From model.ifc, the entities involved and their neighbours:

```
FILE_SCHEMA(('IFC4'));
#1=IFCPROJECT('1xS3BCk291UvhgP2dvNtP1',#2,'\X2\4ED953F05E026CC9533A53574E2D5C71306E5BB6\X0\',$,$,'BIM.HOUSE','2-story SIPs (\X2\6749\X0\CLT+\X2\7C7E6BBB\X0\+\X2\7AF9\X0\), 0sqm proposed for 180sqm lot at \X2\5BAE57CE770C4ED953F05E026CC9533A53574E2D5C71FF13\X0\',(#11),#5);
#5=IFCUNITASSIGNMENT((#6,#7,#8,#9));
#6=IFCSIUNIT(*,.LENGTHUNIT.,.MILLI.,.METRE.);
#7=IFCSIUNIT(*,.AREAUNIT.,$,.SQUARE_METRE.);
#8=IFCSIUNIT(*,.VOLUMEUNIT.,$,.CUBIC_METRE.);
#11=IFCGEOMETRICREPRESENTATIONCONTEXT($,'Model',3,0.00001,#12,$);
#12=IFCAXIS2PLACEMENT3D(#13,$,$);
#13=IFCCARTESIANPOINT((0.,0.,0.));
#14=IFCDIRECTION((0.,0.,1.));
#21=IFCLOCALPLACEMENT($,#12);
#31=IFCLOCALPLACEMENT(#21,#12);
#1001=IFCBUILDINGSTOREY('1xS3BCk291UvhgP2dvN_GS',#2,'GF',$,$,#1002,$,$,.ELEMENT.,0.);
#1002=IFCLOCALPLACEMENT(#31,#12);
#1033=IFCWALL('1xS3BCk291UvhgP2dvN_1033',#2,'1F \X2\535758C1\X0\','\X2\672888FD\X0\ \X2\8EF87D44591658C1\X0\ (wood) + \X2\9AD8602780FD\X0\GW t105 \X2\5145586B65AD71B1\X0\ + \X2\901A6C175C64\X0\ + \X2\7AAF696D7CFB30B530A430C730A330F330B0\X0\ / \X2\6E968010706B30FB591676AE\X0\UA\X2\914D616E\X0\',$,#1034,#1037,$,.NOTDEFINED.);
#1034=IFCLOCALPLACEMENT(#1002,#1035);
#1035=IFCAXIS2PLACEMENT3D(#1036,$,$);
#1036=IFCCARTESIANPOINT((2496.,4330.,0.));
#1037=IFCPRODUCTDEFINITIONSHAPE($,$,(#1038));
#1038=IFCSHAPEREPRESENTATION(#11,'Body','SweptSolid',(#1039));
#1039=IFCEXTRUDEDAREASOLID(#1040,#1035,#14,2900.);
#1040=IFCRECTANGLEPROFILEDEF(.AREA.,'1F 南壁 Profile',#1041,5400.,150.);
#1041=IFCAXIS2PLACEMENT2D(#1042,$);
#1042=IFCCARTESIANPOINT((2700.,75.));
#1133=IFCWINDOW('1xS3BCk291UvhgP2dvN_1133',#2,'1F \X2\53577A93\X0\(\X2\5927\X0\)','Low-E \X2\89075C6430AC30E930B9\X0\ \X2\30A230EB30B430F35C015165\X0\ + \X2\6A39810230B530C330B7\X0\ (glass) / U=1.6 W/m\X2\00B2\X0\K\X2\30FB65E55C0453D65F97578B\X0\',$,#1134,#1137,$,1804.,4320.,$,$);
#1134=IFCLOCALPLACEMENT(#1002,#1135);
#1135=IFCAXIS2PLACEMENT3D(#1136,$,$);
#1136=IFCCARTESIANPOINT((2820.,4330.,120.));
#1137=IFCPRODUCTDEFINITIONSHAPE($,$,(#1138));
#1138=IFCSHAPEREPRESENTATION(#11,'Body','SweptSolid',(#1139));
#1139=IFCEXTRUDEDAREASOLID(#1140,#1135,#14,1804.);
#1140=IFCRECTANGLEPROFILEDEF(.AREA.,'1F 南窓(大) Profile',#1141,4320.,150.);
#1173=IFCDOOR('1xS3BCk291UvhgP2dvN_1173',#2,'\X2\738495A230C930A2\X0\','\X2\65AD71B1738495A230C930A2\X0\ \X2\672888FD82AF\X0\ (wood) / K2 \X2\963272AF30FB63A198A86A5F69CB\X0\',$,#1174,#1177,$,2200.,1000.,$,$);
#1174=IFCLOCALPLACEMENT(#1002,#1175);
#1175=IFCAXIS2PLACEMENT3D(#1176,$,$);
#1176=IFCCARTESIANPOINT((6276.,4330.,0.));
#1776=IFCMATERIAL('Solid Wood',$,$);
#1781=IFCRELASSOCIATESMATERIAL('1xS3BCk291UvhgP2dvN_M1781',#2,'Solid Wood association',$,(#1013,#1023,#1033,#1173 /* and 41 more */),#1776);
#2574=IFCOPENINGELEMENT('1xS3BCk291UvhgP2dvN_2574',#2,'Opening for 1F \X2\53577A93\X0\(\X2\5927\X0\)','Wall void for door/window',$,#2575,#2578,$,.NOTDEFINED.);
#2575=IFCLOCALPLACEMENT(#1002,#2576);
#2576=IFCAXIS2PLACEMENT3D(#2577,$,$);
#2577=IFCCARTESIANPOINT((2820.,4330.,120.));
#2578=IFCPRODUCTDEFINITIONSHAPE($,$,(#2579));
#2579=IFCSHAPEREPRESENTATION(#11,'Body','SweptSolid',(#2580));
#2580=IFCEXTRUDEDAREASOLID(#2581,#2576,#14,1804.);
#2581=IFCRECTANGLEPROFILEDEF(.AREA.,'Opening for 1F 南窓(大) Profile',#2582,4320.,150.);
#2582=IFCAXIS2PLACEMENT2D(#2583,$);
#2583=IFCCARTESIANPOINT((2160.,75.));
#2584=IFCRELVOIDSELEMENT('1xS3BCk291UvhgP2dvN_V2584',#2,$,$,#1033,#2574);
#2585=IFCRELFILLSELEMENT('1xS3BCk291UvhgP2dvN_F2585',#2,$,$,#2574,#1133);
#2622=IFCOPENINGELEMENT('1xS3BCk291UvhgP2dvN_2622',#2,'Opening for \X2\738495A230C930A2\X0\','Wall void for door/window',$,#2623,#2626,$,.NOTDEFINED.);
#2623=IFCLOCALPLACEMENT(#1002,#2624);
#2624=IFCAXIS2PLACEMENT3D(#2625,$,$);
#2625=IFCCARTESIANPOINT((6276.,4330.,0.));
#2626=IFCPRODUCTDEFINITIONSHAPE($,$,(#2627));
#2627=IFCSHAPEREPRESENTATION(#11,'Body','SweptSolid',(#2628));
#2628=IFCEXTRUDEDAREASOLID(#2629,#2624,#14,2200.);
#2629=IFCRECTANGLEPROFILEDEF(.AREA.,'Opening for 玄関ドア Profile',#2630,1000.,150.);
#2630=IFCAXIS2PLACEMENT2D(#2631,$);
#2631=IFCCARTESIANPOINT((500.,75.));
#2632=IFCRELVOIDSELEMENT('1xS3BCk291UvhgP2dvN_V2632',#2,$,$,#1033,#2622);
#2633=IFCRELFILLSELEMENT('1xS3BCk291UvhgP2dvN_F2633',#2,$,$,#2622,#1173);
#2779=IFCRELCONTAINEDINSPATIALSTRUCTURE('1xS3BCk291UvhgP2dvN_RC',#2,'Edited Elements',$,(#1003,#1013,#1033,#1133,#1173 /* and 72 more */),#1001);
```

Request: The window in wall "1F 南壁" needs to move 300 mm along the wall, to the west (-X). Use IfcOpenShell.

```python
import ifcopenshell
import ifcopenshell.api.geometry
import ifcopenshell.util.placement

model = ifcopenshell.open("model.ifc")

window = model.by_id(1133)
opening = window.FillsVoids[0].RelatingOpeningElement
wall = opening.VoidsElements[0].RelatingBuildingElement

wall_matrix = ifcopenshell.util.placement.get_local_placement(wall.ObjectPlacement)
shift = wall_matrix[:3, 0] * -300.0
before = ifcopenshell.util.placement.get_local_placement(window.ObjectPlacement)[:3, 3].copy()

# The window is not placed relative to its opening, so move both.
for product in (opening, window):
    matrix = ifcopenshell.util.placement.get_local_placement(product.ObjectPlacement)
    matrix[:3, 3] += shift
    ifcopenshell.api.geometry.edit_object_placement(model, product=product, matrix=matrix, is_si=False)

after = ifcopenshell.util.placement.get_local_placement(window.ObjectPlacement)[:3, 3]
print("window moved by", (after - before).round(3) + 0.0)

model.write("model_v2.ifc")
```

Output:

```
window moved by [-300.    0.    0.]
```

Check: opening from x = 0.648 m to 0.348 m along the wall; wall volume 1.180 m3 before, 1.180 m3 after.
